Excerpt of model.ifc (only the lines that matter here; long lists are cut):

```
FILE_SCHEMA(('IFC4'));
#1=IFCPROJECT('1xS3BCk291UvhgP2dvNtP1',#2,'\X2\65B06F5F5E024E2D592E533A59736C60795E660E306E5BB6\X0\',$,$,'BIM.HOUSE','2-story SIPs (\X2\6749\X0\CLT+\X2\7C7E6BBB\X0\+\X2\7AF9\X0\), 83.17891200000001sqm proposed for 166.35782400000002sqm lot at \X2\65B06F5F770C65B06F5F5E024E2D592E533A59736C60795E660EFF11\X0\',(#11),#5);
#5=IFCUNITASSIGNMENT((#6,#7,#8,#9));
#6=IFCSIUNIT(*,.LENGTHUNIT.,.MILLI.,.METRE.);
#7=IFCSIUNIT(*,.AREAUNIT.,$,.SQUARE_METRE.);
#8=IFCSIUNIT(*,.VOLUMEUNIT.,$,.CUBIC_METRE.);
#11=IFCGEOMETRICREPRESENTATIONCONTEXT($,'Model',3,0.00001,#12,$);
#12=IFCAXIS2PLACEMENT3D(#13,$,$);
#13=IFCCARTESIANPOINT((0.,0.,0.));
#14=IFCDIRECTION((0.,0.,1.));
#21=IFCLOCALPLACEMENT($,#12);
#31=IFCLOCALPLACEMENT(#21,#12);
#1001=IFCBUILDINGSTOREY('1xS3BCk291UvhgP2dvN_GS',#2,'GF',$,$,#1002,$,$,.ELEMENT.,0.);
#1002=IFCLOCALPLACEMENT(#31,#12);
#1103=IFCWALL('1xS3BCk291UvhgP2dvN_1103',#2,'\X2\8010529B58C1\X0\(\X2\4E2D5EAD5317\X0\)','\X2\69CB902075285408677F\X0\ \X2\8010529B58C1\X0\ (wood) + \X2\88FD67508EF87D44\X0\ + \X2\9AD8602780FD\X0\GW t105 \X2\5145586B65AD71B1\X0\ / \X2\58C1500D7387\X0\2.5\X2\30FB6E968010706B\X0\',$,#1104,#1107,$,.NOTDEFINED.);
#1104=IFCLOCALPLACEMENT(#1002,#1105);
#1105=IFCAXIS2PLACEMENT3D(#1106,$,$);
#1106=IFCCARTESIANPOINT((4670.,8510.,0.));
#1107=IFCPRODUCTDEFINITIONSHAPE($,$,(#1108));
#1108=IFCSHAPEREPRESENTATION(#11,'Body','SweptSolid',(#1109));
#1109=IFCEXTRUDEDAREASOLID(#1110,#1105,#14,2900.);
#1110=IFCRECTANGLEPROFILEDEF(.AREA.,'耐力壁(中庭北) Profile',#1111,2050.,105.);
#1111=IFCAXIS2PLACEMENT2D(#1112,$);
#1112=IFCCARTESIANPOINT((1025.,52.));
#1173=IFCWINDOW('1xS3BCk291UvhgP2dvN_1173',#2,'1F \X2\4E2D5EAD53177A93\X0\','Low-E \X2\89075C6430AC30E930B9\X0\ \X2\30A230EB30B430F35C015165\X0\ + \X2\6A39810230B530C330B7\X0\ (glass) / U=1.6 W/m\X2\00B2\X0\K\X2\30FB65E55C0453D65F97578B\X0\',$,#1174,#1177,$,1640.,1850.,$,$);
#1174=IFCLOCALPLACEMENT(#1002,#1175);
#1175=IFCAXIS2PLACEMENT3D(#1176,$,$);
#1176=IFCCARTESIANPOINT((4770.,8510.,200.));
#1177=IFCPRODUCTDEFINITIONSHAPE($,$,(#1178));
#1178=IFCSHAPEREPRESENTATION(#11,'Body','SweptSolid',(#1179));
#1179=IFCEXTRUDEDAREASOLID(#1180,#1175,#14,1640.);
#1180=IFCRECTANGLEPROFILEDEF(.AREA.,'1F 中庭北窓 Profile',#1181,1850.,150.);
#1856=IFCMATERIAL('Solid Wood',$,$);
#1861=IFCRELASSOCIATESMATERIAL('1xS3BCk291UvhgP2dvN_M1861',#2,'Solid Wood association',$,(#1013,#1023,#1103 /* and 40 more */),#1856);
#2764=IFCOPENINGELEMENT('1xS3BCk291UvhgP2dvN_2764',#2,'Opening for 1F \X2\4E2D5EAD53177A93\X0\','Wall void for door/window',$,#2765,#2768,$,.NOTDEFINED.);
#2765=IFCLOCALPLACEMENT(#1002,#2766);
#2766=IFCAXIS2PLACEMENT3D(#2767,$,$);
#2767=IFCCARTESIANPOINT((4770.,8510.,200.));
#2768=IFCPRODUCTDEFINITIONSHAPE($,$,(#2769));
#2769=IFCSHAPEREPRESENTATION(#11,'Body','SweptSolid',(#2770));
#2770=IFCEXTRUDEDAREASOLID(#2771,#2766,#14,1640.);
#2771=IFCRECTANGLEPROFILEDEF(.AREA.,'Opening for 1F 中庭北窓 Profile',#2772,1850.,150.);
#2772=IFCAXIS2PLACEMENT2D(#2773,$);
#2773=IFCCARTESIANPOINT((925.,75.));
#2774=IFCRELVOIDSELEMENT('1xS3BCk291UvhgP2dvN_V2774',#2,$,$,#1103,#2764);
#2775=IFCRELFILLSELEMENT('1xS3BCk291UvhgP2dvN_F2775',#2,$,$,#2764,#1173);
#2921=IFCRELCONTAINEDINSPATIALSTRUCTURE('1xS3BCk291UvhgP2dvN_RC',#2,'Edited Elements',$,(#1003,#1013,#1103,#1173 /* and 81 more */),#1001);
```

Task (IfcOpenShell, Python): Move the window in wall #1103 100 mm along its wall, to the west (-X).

```python
import ifcopenshell
import ifcopenshell.api.geometry
import ifcopenshell.util.placement

model = ifcopenshell.open("model.ifc")

window = model.by_guid("1xS3BCk291UvhgP2dvN_1173")
opening = window.FillsVoids[0].RelatingOpeningElement
wall = opening.VoidsElements[0].RelatingBuildingElement

wall_matrix = ifcopenshell.util.placement.get_local_placement(wall.ObjectPlacement)
shift = wall_matrix[:3, 0] * -100.0
before = ifcopenshell.util.placement.get_local_placement(window.ObjectPlacement)[:3, 3].copy()

# The window is not placed relative to its opening, so move both.
for product in (opening, window):
    matrix = ifcopenshell.util.placement.get_local_placement(product.ObjectPlacement)
    matrix[:3, 3] += shift
    ifcopenshell.api.geometry.edit_object_placement(model, product=product, matrix=matrix, is_si=False)

after = ifcopenshell.util.placement.get_local_placement(window.ObjectPlacement)[:3, 3]
print("window moved by", (after - before).round(3) + 0.0)

model.write("model_rev.ifc")
```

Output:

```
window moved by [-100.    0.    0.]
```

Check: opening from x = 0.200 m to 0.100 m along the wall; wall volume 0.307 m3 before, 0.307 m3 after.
